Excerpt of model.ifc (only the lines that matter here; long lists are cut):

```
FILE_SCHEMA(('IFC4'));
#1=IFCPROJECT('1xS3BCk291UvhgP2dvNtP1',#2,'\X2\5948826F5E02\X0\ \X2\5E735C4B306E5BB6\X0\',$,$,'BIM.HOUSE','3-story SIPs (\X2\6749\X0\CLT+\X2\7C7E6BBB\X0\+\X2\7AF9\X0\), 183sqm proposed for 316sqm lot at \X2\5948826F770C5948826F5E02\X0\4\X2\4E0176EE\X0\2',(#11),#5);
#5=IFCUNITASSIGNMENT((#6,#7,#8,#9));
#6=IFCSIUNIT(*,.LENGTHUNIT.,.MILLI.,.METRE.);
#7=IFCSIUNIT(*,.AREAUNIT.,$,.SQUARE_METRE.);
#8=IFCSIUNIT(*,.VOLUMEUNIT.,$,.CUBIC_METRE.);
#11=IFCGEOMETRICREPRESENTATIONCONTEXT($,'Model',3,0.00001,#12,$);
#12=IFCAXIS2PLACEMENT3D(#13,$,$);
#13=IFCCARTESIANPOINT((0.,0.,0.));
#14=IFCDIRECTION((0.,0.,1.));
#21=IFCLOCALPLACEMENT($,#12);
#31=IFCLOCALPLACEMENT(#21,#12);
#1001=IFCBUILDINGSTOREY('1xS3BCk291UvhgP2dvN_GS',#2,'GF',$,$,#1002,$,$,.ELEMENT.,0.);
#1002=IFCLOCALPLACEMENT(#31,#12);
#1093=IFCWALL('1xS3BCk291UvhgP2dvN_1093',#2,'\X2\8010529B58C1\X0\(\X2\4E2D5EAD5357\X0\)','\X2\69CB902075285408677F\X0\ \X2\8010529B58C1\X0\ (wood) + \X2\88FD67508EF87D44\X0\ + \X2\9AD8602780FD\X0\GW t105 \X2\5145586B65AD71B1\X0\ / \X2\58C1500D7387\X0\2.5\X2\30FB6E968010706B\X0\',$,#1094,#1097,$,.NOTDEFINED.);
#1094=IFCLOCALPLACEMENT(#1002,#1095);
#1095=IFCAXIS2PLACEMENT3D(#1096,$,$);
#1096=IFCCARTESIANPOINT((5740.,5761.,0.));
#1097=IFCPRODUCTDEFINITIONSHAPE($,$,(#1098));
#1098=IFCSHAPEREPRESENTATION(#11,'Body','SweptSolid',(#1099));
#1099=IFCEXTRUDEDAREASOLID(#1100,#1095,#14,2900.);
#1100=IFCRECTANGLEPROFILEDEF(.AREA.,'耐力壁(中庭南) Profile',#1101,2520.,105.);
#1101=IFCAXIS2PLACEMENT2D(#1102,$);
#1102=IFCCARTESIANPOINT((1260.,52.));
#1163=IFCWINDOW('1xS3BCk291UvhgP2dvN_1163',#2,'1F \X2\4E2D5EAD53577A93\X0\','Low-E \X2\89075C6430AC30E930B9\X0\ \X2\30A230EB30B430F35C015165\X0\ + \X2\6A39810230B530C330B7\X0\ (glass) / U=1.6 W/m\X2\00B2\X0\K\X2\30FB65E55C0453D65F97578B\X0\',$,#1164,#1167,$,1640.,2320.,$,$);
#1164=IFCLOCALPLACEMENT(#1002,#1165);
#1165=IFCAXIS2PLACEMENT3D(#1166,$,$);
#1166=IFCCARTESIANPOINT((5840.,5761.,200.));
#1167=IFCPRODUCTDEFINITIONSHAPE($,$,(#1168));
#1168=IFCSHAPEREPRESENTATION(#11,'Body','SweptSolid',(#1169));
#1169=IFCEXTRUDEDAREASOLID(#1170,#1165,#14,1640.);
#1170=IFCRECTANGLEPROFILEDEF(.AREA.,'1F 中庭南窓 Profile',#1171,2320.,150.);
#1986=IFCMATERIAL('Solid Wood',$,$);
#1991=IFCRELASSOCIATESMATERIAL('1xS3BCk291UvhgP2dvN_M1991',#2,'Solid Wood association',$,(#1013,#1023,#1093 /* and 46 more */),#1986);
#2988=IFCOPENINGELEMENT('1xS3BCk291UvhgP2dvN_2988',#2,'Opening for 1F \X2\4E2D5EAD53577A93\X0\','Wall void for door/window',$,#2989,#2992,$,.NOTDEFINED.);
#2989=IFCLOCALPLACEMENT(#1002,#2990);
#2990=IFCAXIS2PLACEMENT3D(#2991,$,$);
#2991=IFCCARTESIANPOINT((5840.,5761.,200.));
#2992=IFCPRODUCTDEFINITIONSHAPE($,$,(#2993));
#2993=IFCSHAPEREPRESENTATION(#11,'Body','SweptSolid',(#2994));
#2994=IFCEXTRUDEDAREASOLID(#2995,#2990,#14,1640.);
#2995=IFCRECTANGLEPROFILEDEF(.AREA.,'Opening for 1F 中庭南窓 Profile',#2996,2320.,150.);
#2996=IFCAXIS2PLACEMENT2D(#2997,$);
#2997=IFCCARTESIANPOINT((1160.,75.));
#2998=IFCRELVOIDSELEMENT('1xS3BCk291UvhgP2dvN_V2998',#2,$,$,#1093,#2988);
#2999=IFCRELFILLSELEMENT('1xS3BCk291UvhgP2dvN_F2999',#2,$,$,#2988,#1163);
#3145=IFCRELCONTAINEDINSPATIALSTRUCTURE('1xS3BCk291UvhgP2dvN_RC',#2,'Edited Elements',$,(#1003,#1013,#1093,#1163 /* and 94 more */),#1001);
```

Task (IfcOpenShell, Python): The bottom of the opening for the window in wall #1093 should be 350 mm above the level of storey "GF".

```python
import numpy as np
import ifcopenshell
import ifcopenshell.api.geometry
import ifcopenshell.geom
import ifcopenshell.util.element
import ifcopenshell.util.placement
import ifcopenshell.util.shape
import ifcopenshell.util.unit

model = ifcopenshell.open("model.ifc")
unit_scale = ifcopenshell.util.unit.calculate_unit_scale(model)

window = model.by_id(1163)
opening = window.FillsVoids[0].RelatingOpeningElement
storey = ifcopenshell.util.element.get_container(window, ifc_class="IfcBuildingStorey")
level = ifcopenshell.util.placement.get_local_placement(storey.ObjectPlacement)[2, 3]

# The opening's origin need not be at the sill, so measure its lowest point.
shape = ifcopenshell.geom.create_shape(ifcopenshell.geom.settings(), opening)
bottom = ifcopenshell.util.shape.get_shape_bottom_elevation(shape, shape.geometry) / unit_scale
dz = level + 0.35 / unit_scale - bottom

shift = np.array([0.0, 0.0, dz])
# The window is not placed relative to its opening, so move both.
for product in (opening, window):
    matrix = ifcopenshell.util.placement.get_local_placement(product.ObjectPlacement)
    matrix[:3, 3] += shift
    ifcopenshell.api.geometry.edit_object_placement(model, product=product, matrix=matrix, is_si=False)

print(f"moved by {dz * unit_scale:+.3f} m")

model.write("model-out.ifc")
```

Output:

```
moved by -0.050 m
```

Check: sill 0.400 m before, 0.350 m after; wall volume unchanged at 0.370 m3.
